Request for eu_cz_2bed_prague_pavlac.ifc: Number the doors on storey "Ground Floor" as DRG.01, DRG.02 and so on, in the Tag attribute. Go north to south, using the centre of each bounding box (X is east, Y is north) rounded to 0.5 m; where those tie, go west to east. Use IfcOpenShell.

First a look at what the model holds.

```python
import ifcopenshell
import ifcopenshell.util.element
import ifcopenshell.util.placement

model = ifcopenshell.open("eu_cz_2bed_prague_pavlac.ifc")
print(model.schema)
storey = next(s for s in model.by_type("IfcBuildingStorey") if s.Name == "Ground Floor")
doors = [e for e in ifcopenshell.util.element.get_decomposition(storey) if e.is_a("IfcDoor")]
for e in sorted(doors, key=lambda e: e.id()):
    origin = ifcopenshell.util.placement.get_local_placement(e.ObjectPlacement)[:3, 3]
    print(e.id(), e.Tag, e.Name, origin.round(2) + 0.0, sep=" | ")
```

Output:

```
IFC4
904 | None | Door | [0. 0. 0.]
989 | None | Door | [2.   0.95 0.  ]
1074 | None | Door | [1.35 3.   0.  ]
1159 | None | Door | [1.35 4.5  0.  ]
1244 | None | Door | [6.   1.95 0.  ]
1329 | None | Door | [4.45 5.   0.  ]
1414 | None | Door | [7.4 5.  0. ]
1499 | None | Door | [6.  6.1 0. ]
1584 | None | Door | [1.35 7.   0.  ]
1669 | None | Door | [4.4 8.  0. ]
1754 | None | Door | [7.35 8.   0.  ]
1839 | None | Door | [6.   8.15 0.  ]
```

```python
import ifcopenshell
import ifcopenshell.geom
import ifcopenshell.util.element
import ifcopenshell.util.shape

model = ifcopenshell.open("eu_cz_2bed_prague_pavlac.ifc")
settings = ifcopenshell.geom.settings()
settings.set("use-world-coords", True)


def centre(element):
    shape = ifcopenshell.geom.create_shape(settings, element)
    return ifcopenshell.util.shape.get_bbox_centroid(shape.geometry)


storey = next(s for s in model.by_type("IfcBuildingStorey") if s.Name == "Ground Floor")
doors = [e for e in ifcopenshell.util.element.get_decomposition(storey) if e.is_a("IfcDoor")]

# Insertion points can sit at a corner or the storey origin, so sort by the geometry (in metres).
centres = {e: centre(e) for e in doors}
doors.sort(key=lambda e: (-round(centres[e][1] / 0.5), centres[e][0]))

for i, e in enumerate(doors, start=1):
    number = f"DRG.{i:02d}"
    e.Tag = number
    print(e.id(), number)

model.write("eu_cz_2bed_prague_pavlac_updated.ifc")
```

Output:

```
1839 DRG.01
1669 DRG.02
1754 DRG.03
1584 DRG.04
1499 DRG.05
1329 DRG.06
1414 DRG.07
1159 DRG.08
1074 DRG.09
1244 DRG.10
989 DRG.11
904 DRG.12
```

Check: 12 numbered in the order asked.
